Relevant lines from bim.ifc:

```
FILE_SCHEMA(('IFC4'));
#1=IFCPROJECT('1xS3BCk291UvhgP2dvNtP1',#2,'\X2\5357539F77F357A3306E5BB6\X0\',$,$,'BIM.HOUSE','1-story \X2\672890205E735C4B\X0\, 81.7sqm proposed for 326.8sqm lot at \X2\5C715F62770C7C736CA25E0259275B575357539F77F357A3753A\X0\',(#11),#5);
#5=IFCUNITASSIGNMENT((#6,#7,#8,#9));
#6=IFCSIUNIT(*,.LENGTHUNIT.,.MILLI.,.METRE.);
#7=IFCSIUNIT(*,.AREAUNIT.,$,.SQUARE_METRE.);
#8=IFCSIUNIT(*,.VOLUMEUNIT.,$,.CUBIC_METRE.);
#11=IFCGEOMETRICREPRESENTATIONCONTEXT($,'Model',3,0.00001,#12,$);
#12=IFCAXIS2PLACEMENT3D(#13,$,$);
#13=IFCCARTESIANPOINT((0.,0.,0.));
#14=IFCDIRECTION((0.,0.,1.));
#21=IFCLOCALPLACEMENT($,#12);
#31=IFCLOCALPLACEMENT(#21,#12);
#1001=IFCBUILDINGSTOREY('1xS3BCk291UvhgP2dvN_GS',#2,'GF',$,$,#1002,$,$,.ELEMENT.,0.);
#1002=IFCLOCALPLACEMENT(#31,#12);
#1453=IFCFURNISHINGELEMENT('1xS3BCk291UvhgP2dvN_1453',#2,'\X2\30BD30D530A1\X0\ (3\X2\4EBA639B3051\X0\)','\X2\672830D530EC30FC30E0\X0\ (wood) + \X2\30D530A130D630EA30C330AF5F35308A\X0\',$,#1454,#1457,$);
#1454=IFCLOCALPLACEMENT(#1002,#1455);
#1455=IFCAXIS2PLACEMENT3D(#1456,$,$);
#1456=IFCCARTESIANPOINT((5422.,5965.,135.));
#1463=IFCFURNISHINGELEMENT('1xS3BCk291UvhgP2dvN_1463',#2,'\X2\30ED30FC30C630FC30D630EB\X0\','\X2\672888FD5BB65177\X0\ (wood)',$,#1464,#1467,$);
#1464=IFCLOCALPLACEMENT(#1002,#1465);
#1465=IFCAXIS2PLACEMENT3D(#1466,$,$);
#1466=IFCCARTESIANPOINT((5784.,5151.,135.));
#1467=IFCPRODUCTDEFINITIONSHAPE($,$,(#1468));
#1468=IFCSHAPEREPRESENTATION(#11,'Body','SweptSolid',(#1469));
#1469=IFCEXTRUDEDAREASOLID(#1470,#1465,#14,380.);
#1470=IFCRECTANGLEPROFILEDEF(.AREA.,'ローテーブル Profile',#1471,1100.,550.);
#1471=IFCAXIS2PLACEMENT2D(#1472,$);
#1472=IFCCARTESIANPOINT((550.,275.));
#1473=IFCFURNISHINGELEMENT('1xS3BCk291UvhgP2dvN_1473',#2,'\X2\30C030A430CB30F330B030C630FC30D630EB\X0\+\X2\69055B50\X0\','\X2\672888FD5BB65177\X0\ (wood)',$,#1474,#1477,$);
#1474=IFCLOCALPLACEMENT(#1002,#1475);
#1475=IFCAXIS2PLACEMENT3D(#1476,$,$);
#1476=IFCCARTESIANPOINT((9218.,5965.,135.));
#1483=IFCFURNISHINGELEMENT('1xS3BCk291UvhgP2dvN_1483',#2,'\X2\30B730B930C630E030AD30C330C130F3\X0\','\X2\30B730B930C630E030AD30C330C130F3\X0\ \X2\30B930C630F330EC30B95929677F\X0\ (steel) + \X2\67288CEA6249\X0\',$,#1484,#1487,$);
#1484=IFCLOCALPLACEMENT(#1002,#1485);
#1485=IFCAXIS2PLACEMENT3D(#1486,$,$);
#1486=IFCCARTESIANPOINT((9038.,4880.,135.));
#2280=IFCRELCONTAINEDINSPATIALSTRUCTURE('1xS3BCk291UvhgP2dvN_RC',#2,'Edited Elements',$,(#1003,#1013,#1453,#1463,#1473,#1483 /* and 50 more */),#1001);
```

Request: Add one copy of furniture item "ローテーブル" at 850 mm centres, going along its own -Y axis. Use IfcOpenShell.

```python
import ifcopenshell
import ifcopenshell.api.geometry
import ifcopenshell.api.root
import ifcopenshell.util.element
import ifcopenshell.util.placement
import ifcopenshell.util.unit

model = ifcopenshell.open("bim.ifc")
unit_scale = ifcopenshell.util.unit.calculate_unit_scale(model)


def reuse_history(source, copy):
    """copy_class also copies each property set's owner history, people and application; keep the originals."""
    for rel in copy.IsDefinedBy:
        if rel.is_a("IfcRelDefinesByProperties") and (history := rel.RelatingPropertyDefinition.OwnerHistory):
            rel.RelatingPropertyDefinition.OwnerHistory = source.OwnerHistory
            ifcopenshell.util.element.remove_deep2(model, history)


source = model.by_id(1463)
base = ifcopenshell.util.placement.get_local_placement(source.ObjectPlacement)
step = -base[:3, 1] * 0.85 / unit_scale

for i in range(1, 2):
    copy = ifcopenshell.api.root.copy_class(model, product=source)
    copy.Representation = ifcopenshell.util.element.copy_deep(
        model, source.Representation, exclude=["IfcGeometricRepresentationContext", "IfcRepresentationMap"]
    )
    reuse_history(source, copy)
    matrix = base.copy()
    matrix[:3, 3] += i * step
    print("added at", matrix[:3, 3].round(3) + 0.0)
    ifcopenshell.api.geometry.edit_object_placement(model, product=copy, matrix=matrix, is_si=False)

model.write("bim_edited.ifc")
```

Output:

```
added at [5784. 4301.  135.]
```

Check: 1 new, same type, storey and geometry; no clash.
